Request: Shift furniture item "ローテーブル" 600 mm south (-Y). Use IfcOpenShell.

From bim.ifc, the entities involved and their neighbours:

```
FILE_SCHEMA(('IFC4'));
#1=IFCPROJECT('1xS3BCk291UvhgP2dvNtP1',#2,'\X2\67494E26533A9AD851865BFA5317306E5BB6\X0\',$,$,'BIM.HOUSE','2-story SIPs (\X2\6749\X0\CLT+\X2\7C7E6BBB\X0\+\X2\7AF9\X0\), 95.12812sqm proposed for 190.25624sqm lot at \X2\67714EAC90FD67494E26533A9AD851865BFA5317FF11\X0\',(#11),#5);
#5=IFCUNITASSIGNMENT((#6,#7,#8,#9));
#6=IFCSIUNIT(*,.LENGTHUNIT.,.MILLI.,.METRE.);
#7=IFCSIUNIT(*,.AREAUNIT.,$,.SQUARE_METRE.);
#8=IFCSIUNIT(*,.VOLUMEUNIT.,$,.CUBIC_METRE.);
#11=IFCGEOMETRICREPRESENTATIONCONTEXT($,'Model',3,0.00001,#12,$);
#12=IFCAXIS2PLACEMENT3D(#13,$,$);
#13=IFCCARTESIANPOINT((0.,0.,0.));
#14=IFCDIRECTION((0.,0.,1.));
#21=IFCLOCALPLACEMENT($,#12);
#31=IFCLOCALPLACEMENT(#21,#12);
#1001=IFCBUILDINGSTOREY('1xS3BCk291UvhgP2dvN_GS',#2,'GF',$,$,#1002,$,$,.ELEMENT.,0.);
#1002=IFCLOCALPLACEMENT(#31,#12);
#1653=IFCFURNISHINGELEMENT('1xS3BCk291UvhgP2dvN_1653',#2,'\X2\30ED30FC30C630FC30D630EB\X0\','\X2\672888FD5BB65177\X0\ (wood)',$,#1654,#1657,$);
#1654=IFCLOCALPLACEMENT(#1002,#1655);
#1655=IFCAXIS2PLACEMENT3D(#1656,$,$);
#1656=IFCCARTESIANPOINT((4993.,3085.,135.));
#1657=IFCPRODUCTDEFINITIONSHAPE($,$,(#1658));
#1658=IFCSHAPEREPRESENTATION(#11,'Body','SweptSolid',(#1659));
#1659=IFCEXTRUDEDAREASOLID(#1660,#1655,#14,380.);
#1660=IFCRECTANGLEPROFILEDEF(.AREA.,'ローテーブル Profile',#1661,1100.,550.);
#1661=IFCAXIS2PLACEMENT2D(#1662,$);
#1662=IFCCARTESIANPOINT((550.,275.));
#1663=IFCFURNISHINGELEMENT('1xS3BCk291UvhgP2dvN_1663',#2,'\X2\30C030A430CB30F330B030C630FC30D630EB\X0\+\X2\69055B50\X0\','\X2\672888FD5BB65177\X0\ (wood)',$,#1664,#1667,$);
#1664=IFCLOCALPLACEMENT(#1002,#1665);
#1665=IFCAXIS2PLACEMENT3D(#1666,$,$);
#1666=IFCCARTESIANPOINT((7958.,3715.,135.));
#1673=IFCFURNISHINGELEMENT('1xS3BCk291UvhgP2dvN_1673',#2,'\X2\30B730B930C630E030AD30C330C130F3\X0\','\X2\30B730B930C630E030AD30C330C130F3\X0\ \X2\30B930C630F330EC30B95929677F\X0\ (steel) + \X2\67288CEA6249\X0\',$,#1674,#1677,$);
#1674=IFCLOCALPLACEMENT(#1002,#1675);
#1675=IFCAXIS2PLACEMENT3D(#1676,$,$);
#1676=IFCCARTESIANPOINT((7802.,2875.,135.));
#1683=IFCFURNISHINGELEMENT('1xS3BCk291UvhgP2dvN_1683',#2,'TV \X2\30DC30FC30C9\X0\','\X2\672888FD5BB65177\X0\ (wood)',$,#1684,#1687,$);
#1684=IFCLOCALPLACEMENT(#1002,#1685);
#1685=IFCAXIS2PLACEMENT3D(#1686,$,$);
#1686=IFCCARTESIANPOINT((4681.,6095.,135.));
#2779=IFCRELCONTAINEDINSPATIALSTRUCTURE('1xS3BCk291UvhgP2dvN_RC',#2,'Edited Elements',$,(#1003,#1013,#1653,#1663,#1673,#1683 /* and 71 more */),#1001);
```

```python
import ifcopenshell
import ifcopenshell.api.geometry
import ifcopenshell.util.placement

model = ifcopenshell.open("bim.ifc")

item = model.by_guid("1xS3BCk291UvhgP2dvN_1653")
matrix = ifcopenshell.util.placement.get_local_placement(item.ObjectPlacement)
matrix[1, 3] -= 600.0
ifcopenshell.api.geometry.edit_object_placement(model, product=item, matrix=matrix, is_si=False)

print(ifcopenshell.util.placement.get_local_placement(item.ObjectPlacement).round(3) + 0.0)

model.write("bim_edited.ifc")
```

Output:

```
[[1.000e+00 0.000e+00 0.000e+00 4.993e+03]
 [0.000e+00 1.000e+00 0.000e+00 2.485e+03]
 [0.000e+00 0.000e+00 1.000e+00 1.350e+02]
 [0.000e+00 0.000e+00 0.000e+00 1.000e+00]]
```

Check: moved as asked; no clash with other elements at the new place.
